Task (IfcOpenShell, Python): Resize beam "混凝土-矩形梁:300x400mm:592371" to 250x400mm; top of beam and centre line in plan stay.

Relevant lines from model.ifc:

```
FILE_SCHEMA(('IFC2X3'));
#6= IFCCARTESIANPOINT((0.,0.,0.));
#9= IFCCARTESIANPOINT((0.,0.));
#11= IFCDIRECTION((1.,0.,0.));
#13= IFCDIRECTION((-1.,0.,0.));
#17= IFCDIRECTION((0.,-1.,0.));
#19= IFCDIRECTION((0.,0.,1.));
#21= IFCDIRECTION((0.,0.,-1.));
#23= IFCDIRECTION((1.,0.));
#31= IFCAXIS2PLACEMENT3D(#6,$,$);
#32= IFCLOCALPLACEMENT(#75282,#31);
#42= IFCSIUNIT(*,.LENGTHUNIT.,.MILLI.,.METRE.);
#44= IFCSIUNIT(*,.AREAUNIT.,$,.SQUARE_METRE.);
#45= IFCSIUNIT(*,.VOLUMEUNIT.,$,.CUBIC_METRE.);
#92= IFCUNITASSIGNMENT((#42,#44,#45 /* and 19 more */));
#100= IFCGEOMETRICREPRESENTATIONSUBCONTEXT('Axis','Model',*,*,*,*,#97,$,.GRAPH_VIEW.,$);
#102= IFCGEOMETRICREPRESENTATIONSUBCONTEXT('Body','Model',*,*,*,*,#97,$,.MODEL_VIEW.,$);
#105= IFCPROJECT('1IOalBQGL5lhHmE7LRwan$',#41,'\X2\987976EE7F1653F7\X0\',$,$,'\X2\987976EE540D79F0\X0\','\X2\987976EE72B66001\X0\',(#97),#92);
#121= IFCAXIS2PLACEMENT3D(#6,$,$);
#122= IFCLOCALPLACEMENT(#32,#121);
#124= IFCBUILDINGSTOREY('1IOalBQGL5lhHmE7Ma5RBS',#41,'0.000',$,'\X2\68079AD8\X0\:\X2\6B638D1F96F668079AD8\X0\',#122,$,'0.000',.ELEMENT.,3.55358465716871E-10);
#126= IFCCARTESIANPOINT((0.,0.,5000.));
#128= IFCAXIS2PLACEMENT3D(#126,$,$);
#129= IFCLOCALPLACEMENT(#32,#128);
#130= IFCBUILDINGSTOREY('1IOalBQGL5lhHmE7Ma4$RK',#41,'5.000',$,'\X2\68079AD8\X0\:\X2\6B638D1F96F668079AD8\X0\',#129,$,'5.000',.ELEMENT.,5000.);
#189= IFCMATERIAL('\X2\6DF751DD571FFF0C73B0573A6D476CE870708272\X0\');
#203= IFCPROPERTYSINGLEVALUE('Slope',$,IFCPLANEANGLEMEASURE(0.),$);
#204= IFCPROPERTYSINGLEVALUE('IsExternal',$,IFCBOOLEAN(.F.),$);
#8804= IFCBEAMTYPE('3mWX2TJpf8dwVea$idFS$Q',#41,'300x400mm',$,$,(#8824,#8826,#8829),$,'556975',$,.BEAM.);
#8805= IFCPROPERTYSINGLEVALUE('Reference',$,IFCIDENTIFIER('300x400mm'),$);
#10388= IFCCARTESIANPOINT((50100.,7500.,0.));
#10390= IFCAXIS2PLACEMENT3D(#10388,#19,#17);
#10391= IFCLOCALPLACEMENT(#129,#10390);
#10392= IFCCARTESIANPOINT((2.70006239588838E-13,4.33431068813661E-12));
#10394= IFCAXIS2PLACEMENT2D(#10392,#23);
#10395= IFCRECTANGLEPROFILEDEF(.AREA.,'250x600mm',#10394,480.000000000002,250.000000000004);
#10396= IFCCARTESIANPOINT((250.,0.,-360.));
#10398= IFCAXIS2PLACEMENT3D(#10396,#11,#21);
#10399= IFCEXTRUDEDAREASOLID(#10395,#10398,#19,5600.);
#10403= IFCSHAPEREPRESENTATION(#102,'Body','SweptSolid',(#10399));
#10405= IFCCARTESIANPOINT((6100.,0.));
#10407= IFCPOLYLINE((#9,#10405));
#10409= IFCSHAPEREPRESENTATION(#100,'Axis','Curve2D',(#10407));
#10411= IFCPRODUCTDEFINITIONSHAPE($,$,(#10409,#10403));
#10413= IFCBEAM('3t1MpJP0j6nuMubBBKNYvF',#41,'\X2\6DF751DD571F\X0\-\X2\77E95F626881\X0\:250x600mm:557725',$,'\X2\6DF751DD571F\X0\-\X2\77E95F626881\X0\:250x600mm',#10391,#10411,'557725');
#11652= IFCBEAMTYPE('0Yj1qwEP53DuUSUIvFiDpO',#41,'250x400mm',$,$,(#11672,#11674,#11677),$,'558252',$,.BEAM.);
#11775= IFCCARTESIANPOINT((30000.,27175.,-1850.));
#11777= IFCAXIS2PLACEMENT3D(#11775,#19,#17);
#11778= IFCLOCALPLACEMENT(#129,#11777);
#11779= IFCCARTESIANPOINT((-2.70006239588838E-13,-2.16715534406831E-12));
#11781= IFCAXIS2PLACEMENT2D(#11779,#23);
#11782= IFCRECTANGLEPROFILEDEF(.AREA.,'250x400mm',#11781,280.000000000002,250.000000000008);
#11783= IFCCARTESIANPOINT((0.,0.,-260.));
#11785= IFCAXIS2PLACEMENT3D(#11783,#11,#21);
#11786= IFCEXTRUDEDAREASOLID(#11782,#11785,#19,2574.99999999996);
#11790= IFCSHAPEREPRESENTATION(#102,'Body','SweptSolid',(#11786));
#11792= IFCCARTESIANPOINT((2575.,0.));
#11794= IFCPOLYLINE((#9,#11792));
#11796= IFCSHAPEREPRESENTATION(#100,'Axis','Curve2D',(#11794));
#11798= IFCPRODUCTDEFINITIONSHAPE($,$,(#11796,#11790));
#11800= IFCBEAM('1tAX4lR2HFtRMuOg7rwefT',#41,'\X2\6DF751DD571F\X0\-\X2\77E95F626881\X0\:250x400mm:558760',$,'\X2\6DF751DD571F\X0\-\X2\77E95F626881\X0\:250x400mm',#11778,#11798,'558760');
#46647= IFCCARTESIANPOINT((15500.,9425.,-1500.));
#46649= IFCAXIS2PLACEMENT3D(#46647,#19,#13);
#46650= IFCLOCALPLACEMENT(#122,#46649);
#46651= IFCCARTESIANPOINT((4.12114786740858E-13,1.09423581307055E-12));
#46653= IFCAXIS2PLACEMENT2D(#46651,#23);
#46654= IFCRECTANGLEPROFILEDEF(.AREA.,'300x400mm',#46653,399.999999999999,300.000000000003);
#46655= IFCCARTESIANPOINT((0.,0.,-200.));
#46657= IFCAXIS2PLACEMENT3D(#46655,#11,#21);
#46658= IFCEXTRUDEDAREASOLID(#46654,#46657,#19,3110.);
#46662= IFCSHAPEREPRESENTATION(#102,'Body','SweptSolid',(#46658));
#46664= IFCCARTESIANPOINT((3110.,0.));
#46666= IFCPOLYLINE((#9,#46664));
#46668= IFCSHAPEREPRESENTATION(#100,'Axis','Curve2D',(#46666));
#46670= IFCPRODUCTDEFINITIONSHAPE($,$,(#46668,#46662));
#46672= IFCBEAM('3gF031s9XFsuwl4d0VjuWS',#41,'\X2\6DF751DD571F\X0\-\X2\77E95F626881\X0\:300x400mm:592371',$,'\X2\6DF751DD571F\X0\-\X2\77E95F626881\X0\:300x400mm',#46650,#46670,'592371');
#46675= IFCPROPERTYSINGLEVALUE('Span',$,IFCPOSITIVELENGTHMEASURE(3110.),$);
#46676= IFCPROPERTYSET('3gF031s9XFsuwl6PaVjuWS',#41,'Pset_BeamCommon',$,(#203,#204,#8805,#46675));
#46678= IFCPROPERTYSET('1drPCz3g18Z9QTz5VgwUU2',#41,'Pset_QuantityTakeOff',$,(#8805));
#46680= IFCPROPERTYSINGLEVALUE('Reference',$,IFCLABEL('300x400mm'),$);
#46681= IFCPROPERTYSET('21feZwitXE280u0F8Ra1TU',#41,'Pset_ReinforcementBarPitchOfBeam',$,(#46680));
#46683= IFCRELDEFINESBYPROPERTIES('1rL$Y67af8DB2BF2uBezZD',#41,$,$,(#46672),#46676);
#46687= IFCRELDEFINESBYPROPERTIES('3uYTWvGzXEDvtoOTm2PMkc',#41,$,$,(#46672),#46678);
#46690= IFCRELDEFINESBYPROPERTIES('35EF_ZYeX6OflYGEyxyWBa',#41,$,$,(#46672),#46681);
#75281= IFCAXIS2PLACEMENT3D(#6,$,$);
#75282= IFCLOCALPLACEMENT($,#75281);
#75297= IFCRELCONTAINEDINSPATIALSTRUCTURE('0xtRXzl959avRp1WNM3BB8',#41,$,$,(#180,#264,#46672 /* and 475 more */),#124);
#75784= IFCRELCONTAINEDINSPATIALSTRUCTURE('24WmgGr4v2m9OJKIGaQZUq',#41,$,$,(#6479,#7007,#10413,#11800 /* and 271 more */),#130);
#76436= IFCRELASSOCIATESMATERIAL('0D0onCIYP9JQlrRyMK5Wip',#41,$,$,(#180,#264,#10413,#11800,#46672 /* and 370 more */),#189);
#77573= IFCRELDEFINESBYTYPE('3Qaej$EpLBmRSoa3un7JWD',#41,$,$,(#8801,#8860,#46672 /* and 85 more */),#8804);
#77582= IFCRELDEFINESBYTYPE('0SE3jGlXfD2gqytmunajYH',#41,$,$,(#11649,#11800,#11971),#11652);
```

```python
import ifcopenshell
import ifcopenshell.api.pset
import ifcopenshell.api.type
import ifcopenshell.util.element
import ifcopenshell.util.representation

model = ifcopenshell.open("model.ifc")

member = model.by_id(46672)
source = next(p for p in model.by_type("IfcRectangleProfileDef") if p.ProfileName == "250x400mm")

body = ifcopenshell.util.representation.get_representation(member, "Model", "Body")
solid = body.Items[0]
old_profile = solid.SweptArea

# Copy the section's sizes but keep this member's own profile position.
profile = ifcopenshell.util.element.copy(model, source)
# Profiles are centred, so shift by half the change in depth to hold the top.
shift = (old_profile.XDim - profile.XDim) / 2
x, y = old_profile.Position.Location.Coordinates
up = (-1.0, 0.0)  # upwards, in the solid's own plane
location = model.createIfcCartesianPoint((x + up[0] * shift, y + up[1] * shift))
profile.Position = model.createIfcAxis2Placement2D(location, old_profile.Position.RefDirection)
solid.SweptArea = profile
if not model.get_total_inverses(old_profile):
    ifcopenshell.util.element.remove_deep2(model, old_profile)

new_type = model.by_guid("0Yj1qwEP53DuUSUIvFiDpO")
ifcopenshell.api.type.assign_type(
    model, related_objects=[member], relating_type=new_type, should_map_representations=False
)
member.Name = member.Name.replace("300x400mm", "250x400mm")
member.ObjectType = "混凝土-矩形梁:250x400mm"
pset = model.by_id(ifcopenshell.util.element.get_pset(member, "Pset_BeamCommon", should_inherit=False)["id"])
ifcopenshell.api.pset.edit_pset(model, pset=pset, properties={"Reference": "250x400mm"})
pset = model.by_id(ifcopenshell.util.element.get_pset(member, "Pset_QuantityTakeOff", should_inherit=False)["id"])
ifcopenshell.api.pset.edit_pset(model, pset=pset, properties={"Reference": "250x400mm"})
pset = model.by_id(ifcopenshell.util.element.get_pset(member, "Pset_ReinforcementBarPitchOfBeam", should_inherit=False)["id"])
ifcopenshell.api.pset.edit_pset(model, pset=pset, properties={"Reference": "250x400mm"})

print(solid.SweptArea)

model.write("model_v2.ifc")
```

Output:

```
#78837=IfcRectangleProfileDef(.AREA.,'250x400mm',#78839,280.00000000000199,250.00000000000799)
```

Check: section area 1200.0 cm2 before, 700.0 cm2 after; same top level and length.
